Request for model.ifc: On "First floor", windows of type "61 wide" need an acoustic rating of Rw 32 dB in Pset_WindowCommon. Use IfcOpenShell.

First a look at what the model holds.

```python
import ifcopenshell
import ifcopenshell.util.element

model = ifcopenshell.open("model.ifc")
print(model.schema)
storey = next(s for s in model.by_type("IfcBuildingStorey") if s.Name == "First floor")
windows = [e for e in ifcopenshell.util.element.get_decomposition(storey) if e.is_a("IfcWindow")]
seen = {}
for e in windows:
    element_type = ifcopenshell.util.element.get_type(e)
    key = (element_type.Name if element_type != e and element_type else None, ifcopenshell.util.element.get_pset(e, "Pset_WindowCommon", "AcousticRating"))
    seen[key] = seen.get(key, 0) + 1
for (name, value), count in sorted(seen.items(), key=str):
    print(count, "x", name, "|", value)
```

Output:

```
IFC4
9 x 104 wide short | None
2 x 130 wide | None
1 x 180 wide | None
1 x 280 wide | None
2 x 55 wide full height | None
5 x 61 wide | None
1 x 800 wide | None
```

```python
import ifcopenshell
import ifcopenshell.api.pset
import ifcopenshell.util.element

model = ifcopenshell.open("model.ifc")

storey = next(s for s in model.by_type("IfcBuildingStorey") if s.Name == "First floor")
windows = [e for e in ifcopenshell.util.element.get_decomposition(storey) if e.is_a("IfcWindow")]

count = 0
for e in windows:
    element_type = ifcopenshell.util.element.get_type(e)
    if element_type in (None, e) or element_type.Name != "61 wide":
        continue
    # add_pset returns the element's existing set when there is one.
    pset = ifcopenshell.api.pset.add_pset(model, product=e, name="Pset_WindowCommon")
    ifcopenshell.api.pset.edit_pset(model, pset=pset, properties={"AcousticRating": "Rw 32 dB"})
    count += 1

print(count, "windows updated")

model.write("model_edited.ifc")
```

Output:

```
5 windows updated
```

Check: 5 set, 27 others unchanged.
